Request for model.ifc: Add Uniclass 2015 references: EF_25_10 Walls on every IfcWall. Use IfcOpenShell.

First a look at what the model holds.

```python
import ifcopenshell

model = ifcopenshell.open("model.ifc")
print(model.schema)
print("classifications:", [c.Name for c in model.by_type("IfcClassification")])
for ifc_class in ("IfcDoor", "IfcRoof", "IfcStair", "IfcWall", "IfcWindow"):
    print(ifc_class, len(model.by_type(ifc_class)))
```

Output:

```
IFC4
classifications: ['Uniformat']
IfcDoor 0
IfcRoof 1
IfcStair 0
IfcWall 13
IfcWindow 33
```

```python
import ifcopenshell
import ifcopenshell.api.classification

model = ifcopenshell.open("model.ifc")

system = ifcopenshell.api.classification.add_classification(model, classification="Uniclass 2015")

codes = {
    "IfcWall": ("EF_25_10", "Walls"),
}
for ifc_class, (code, name) in codes.items():
    products = model.by_type(ifc_class)
    ifcopenshell.api.classification.add_reference(
        model, products=products, classification=system, identification=code, name=name
    )
    print(code, len(products))

model.write("model_updated.ifc")
```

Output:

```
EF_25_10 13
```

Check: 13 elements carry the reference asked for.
